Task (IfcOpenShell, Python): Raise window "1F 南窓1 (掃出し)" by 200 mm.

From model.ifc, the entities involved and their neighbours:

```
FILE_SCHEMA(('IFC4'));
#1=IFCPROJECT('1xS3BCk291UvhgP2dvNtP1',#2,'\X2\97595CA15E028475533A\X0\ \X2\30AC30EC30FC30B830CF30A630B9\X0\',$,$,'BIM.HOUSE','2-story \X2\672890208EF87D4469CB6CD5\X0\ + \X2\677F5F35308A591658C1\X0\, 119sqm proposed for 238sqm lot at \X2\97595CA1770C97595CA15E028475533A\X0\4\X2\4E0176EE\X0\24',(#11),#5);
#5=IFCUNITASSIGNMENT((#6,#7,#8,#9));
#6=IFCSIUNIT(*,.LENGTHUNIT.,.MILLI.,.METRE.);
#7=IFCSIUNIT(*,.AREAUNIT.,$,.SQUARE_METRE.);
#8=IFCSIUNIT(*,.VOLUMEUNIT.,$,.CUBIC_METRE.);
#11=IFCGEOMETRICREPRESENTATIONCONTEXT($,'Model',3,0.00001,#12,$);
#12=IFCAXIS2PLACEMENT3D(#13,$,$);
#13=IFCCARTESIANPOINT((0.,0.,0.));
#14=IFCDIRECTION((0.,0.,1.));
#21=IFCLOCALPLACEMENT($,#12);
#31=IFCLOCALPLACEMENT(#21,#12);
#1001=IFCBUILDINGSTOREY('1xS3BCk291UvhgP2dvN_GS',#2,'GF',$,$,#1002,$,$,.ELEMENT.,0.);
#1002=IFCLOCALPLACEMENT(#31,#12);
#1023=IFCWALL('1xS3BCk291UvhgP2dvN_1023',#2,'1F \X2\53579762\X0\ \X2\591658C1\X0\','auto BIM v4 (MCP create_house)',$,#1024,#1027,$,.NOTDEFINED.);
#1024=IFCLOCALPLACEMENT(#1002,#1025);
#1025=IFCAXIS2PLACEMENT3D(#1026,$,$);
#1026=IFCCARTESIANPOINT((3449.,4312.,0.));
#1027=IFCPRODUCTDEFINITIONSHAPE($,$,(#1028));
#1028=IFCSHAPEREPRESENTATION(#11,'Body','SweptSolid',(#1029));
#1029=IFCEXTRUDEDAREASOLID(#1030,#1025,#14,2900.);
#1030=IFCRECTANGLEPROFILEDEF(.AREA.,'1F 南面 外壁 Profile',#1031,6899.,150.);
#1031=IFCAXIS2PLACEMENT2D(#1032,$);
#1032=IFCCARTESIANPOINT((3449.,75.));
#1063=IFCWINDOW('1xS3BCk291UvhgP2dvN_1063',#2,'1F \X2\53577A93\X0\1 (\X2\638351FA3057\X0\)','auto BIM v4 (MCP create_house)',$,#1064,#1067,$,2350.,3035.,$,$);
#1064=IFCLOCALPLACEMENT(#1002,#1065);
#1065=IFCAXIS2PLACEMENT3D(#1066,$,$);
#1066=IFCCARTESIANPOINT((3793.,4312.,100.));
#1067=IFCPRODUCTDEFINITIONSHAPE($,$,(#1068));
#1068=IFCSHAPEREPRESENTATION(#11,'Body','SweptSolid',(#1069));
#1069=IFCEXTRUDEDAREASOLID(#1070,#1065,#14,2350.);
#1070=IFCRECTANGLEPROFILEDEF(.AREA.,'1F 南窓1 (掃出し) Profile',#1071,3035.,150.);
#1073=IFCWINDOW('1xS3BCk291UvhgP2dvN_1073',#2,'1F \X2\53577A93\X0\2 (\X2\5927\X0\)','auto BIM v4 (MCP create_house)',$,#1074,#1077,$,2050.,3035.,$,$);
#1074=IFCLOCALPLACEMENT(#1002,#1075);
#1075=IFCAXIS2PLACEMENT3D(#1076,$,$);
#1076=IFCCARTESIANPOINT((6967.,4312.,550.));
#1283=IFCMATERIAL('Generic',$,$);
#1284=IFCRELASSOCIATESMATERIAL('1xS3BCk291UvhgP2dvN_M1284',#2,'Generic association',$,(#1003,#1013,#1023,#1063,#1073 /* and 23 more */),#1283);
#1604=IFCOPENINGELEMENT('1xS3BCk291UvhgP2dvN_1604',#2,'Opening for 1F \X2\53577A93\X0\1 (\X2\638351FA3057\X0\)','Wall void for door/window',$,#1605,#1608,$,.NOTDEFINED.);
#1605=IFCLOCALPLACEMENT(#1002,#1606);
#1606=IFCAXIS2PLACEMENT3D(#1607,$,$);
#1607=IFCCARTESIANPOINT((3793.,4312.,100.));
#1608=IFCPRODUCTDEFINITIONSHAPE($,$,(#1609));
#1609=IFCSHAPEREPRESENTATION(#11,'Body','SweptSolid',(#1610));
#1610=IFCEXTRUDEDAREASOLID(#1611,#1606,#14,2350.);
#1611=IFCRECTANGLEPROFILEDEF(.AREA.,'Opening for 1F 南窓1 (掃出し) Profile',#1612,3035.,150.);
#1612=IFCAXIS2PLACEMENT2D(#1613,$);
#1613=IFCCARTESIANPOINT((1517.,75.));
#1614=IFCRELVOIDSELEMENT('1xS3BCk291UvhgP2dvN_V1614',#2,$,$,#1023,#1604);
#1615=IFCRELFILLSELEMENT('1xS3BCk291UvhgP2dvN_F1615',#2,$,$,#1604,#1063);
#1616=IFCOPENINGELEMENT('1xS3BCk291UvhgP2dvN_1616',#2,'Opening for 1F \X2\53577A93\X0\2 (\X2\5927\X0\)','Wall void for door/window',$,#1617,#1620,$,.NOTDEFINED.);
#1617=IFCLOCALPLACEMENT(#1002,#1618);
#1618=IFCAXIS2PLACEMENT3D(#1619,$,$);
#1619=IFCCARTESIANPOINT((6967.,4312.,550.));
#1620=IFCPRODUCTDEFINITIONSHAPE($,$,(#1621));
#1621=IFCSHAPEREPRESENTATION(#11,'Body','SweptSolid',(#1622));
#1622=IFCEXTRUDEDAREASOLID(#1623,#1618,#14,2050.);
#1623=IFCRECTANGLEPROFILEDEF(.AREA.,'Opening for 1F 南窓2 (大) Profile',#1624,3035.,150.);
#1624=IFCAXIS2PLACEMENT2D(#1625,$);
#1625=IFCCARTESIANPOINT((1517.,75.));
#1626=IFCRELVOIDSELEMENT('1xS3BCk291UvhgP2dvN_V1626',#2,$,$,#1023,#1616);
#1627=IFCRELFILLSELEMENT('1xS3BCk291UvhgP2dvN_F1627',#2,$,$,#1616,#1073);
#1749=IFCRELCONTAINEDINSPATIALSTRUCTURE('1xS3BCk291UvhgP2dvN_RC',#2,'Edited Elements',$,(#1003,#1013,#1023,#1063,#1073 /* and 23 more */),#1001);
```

```python
import numpy as np
import ifcopenshell
import ifcopenshell.api.geometry
import ifcopenshell.util.placement
import ifcopenshell.util.unit

model = ifcopenshell.open("model.ifc")
unit_scale = ifcopenshell.util.unit.calculate_unit_scale(model)

window = model.by_id(1063)
opening = window.FillsVoids[0].RelatingOpeningElement
dz = 200.0

shift = np.array([0.0, 0.0, dz])
# The window is not placed relative to its opening, so move both.
for product in (opening, window):
    matrix = ifcopenshell.util.placement.get_local_placement(product.ObjectPlacement)
    matrix[:3, 3] += shift
    ifcopenshell.api.geometry.edit_object_placement(model, product=product, matrix=matrix, is_si=False)

print(f"moved by {dz * unit_scale:+.3f} m")

model.write("model-out.ifc")
```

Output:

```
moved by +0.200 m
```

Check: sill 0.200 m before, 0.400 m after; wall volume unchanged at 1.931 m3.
